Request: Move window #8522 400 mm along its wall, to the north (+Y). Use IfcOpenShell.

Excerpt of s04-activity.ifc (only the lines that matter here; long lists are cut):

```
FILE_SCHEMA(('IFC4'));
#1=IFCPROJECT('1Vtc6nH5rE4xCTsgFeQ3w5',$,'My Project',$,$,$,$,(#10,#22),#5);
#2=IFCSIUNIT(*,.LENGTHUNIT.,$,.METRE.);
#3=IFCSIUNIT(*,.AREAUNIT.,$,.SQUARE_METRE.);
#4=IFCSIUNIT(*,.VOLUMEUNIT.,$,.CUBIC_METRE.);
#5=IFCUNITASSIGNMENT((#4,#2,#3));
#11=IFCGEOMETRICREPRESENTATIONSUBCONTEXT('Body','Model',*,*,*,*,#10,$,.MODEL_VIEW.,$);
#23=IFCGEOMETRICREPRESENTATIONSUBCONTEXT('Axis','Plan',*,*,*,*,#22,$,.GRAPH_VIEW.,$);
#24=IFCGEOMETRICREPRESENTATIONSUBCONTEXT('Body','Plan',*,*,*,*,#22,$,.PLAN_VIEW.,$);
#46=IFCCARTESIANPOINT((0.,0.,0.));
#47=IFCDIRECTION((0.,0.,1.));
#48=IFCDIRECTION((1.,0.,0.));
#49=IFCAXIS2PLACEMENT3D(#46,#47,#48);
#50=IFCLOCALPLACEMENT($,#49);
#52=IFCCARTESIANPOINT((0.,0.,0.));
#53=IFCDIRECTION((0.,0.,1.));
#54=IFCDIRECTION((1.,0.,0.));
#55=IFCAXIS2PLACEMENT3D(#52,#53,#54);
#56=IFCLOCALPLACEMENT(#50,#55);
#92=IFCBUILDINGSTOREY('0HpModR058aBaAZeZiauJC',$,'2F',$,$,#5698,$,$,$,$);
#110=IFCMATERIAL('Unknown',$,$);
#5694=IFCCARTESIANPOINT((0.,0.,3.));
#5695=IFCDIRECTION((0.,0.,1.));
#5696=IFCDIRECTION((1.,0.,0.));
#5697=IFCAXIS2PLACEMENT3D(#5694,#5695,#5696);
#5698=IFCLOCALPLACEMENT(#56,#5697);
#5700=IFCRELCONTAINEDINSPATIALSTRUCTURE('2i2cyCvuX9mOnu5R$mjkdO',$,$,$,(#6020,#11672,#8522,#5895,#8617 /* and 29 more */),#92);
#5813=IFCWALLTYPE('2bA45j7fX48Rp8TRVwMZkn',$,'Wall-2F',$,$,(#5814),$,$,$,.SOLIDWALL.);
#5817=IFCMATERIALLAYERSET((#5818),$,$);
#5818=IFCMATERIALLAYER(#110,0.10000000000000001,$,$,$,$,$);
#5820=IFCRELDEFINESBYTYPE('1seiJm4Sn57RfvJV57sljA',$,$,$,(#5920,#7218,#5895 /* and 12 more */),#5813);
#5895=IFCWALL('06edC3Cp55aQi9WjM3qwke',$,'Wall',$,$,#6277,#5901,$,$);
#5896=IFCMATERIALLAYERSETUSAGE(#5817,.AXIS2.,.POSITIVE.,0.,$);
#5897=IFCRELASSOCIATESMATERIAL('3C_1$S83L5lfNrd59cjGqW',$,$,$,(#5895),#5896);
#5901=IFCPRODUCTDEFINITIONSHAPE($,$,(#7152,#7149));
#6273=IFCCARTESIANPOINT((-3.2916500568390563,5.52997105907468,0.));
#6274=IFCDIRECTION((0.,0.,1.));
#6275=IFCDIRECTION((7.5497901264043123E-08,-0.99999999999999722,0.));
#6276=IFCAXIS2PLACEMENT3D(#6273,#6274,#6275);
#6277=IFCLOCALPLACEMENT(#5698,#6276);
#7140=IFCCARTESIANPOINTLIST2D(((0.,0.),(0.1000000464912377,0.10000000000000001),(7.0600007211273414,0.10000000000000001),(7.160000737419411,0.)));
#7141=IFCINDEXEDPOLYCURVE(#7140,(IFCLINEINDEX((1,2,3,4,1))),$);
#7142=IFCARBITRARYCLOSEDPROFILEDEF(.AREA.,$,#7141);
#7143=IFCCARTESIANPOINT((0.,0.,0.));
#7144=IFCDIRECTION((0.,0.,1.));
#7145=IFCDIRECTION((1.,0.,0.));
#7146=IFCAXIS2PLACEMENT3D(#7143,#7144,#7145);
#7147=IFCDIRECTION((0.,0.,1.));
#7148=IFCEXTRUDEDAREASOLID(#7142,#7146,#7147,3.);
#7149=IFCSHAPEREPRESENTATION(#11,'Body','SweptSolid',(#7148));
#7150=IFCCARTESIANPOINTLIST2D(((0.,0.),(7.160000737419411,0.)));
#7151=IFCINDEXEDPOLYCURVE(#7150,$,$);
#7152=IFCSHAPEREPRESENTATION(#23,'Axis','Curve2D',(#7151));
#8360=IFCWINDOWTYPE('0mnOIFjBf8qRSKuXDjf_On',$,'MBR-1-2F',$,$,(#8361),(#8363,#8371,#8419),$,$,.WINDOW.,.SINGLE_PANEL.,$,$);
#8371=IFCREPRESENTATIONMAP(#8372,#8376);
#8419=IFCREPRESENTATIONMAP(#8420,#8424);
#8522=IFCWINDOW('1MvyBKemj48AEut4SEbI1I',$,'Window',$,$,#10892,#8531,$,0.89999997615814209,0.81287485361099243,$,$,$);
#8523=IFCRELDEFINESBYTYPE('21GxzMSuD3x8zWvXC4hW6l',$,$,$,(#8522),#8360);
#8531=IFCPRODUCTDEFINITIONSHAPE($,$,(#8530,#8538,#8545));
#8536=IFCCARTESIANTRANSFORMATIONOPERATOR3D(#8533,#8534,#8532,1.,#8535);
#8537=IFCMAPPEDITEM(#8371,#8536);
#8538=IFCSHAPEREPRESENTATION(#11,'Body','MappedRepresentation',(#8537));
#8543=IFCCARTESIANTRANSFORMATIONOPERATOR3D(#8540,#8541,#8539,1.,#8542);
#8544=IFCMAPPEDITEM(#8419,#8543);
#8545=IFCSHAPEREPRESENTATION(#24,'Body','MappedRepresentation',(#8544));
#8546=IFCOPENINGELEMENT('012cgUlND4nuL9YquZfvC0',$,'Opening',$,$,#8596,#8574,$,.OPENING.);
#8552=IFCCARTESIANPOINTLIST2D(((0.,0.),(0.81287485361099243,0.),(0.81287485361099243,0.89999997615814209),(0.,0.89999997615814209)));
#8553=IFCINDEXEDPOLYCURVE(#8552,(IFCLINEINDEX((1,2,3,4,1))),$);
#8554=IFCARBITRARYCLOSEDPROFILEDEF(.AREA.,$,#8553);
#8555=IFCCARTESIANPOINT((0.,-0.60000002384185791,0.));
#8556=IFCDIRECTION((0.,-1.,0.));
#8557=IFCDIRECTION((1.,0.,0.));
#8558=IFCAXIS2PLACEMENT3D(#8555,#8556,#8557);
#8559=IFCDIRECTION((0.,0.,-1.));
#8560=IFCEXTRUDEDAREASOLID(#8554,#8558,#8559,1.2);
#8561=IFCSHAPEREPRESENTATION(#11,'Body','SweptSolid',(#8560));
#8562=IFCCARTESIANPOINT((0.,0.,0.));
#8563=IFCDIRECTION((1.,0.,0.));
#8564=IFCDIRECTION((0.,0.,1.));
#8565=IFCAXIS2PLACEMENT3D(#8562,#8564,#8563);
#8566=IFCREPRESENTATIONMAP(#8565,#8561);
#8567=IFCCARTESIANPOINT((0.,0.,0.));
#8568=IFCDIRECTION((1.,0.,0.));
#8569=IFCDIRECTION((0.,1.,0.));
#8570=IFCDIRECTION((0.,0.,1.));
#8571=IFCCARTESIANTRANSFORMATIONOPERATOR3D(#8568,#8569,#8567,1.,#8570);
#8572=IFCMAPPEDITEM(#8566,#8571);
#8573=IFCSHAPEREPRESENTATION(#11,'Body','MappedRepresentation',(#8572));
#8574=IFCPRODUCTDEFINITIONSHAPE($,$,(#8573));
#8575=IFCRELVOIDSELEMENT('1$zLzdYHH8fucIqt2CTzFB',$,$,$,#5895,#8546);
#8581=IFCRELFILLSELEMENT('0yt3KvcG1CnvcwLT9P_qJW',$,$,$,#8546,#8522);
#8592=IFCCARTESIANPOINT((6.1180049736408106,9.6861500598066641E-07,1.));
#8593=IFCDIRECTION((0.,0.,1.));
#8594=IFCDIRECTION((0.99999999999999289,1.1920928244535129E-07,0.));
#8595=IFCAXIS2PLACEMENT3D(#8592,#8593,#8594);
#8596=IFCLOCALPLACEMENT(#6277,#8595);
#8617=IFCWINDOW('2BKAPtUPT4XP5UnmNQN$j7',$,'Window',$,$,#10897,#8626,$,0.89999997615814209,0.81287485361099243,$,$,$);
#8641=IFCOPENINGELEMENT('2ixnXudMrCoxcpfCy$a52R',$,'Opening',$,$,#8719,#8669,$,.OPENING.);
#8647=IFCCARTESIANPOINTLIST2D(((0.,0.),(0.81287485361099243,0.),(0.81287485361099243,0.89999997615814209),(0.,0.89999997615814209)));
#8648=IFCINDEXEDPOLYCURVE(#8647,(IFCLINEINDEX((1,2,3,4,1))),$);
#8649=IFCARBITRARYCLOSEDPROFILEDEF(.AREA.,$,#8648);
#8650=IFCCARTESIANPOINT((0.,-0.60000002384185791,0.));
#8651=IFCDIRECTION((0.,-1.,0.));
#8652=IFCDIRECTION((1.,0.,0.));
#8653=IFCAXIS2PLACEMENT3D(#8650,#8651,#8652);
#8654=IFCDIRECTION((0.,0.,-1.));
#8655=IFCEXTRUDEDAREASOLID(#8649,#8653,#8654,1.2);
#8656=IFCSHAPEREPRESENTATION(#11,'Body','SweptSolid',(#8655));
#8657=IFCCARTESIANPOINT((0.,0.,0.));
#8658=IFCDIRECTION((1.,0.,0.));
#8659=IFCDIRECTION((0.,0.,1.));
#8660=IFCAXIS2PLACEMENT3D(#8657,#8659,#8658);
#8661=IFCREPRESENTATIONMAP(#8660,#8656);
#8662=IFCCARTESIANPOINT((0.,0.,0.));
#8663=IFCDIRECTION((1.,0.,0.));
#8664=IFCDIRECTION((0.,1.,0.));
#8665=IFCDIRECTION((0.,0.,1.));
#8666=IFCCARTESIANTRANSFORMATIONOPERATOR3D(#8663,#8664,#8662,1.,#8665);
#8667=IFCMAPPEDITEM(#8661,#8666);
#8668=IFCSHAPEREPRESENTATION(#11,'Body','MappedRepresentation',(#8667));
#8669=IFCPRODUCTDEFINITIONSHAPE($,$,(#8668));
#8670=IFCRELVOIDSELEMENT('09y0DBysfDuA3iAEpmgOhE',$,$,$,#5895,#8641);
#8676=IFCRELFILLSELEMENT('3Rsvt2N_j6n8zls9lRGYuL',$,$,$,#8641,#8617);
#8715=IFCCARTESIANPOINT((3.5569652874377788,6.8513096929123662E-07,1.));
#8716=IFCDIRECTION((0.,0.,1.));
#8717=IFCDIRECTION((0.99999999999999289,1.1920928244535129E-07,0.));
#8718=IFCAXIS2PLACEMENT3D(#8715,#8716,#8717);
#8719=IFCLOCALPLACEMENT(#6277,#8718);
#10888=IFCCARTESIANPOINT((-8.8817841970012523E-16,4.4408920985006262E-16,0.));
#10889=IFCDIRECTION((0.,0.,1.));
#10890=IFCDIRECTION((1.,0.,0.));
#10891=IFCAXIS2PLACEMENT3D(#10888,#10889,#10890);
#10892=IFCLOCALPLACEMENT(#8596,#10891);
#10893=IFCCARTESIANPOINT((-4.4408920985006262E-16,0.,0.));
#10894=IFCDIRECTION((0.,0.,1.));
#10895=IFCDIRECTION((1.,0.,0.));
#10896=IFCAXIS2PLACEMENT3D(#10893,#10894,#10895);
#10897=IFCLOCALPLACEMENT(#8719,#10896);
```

```python
import ifcopenshell
import ifcopenshell.api.geometry
import ifcopenshell.util.placement

model = ifcopenshell.open("s04-activity.ifc")

window = model.by_id(8522)
opening = window.FillsVoids[0].RelatingOpeningElement
wall = opening.VoidsElements[0].RelatingBuildingElement

wall_matrix = ifcopenshell.util.placement.get_local_placement(wall.ObjectPlacement)
shift = wall_matrix[:3, 0] * -0.4
before = ifcopenshell.util.placement.get_local_placement(window.ObjectPlacement)[:3, 3].copy()

# The window is placed relative to its opening, so it follows when the opening moves.
matrix = ifcopenshell.util.placement.get_local_placement(opening.ObjectPlacement)
matrix[:3, 3] += shift
ifcopenshell.api.geometry.edit_object_placement(
    model, product=opening, matrix=matrix, is_si=False, should_transform_children=True
)

after = ifcopenshell.util.placement.get_local_placement(window.ObjectPlacement)[:3, 3]
print("window moved by", (after - before).round(3) + 0.0)

model.write("s04-activity-out.ifc")
```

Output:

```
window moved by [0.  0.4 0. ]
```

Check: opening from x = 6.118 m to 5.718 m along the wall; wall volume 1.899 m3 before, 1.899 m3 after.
